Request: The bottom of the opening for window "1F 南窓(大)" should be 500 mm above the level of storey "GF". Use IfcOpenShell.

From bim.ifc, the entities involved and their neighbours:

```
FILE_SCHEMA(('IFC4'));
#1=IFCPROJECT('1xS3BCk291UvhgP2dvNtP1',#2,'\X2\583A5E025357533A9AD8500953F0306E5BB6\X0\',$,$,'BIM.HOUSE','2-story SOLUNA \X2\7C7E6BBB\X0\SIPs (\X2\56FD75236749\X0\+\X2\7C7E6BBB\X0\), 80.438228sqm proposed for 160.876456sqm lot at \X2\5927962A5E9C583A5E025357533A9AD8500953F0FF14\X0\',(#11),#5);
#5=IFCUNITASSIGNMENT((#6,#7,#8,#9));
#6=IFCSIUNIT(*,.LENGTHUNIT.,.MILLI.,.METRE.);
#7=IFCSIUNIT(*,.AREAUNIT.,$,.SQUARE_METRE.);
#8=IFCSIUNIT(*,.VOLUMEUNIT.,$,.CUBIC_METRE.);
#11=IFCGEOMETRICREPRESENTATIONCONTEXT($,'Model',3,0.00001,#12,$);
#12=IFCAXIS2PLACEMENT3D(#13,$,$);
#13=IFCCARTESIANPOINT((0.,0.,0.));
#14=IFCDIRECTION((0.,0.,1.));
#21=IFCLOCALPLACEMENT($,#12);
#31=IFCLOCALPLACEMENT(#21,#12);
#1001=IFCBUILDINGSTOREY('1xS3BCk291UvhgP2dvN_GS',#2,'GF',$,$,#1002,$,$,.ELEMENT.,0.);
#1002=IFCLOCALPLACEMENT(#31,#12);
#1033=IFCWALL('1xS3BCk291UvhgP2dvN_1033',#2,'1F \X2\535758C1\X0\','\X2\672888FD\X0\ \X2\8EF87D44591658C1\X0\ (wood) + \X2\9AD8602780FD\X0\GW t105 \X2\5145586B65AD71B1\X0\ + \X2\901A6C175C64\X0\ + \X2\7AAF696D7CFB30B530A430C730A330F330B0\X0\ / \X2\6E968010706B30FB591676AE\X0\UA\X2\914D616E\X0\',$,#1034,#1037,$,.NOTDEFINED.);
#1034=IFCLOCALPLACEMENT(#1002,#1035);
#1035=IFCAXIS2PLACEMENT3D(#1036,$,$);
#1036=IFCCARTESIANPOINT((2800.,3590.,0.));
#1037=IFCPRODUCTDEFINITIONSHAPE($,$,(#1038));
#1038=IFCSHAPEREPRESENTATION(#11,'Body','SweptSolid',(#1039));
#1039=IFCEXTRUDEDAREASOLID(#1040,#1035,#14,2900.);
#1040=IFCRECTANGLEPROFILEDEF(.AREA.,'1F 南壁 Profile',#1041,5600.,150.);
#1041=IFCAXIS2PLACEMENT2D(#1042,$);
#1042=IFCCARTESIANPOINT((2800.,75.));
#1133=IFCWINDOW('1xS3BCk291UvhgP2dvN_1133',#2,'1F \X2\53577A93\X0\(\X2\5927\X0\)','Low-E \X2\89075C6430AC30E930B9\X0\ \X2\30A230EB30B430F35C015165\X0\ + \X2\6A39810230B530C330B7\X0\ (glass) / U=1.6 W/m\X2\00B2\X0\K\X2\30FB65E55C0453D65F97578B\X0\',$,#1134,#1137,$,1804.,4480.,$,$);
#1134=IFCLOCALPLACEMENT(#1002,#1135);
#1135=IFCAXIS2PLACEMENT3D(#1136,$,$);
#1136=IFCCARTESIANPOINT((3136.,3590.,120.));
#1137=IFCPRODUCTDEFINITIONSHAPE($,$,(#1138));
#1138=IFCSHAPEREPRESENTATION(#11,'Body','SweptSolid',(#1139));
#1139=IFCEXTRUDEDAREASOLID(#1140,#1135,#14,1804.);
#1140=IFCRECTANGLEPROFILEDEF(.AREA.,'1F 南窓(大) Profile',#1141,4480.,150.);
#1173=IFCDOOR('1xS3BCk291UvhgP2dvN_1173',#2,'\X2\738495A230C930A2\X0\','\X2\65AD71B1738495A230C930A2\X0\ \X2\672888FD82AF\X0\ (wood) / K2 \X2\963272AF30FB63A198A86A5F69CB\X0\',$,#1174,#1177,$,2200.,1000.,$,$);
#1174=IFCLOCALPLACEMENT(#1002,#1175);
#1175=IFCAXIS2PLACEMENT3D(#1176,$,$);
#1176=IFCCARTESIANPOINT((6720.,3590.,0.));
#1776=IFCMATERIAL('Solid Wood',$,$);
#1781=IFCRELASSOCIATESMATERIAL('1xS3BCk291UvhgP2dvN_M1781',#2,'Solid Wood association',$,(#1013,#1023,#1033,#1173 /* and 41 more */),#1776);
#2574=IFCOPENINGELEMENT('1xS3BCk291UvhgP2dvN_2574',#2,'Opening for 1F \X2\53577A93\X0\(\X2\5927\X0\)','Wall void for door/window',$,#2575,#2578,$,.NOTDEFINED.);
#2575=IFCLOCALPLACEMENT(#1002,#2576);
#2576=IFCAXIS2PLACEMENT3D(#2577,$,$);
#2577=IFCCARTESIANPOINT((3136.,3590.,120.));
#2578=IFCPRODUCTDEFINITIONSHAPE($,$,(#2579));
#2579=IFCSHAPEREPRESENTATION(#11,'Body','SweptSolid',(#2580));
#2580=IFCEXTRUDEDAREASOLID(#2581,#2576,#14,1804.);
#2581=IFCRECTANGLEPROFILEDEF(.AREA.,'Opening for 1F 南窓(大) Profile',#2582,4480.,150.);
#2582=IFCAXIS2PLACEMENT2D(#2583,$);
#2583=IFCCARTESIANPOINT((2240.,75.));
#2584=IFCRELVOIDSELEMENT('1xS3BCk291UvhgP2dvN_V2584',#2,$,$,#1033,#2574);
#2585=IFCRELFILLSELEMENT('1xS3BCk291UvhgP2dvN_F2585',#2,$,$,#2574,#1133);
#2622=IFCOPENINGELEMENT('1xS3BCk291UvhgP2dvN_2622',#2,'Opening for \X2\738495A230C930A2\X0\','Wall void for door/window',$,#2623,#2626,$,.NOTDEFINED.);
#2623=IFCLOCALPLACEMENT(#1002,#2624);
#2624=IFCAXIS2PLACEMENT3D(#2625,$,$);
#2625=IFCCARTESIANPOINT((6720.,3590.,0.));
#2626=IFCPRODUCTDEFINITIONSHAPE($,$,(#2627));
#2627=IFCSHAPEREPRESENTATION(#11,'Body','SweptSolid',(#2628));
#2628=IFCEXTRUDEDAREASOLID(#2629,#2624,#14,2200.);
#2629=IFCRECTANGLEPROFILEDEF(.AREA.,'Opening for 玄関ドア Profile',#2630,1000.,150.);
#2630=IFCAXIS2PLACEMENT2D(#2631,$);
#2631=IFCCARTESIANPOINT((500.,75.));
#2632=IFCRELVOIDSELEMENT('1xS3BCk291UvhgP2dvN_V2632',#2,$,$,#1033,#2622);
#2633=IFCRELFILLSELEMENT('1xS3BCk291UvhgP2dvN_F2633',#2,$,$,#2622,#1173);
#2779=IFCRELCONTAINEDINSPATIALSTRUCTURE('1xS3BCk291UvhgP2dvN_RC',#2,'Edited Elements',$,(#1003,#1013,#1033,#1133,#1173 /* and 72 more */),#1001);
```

```python
import numpy as np
import ifcopenshell
import ifcopenshell.api.geometry
import ifcopenshell.geom
import ifcopenshell.util.element
import ifcopenshell.util.placement
import ifcopenshell.util.shape
import ifcopenshell.util.unit

model = ifcopenshell.open("bim.ifc")
unit_scale = ifcopenshell.util.unit.calculate_unit_scale(model)

window = model.by_guid("1xS3BCk291UvhgP2dvN_1133")
opening = window.FillsVoids[0].RelatingOpeningElement
storey = ifcopenshell.util.element.get_container(window, ifc_class="IfcBuildingStorey")
level = ifcopenshell.util.placement.get_local_placement(storey.ObjectPlacement)[2, 3]

# The opening's origin need not be at the sill, so measure its lowest point.
shape = ifcopenshell.geom.create_shape(ifcopenshell.geom.settings(), opening)
bottom = ifcopenshell.util.shape.get_shape_bottom_elevation(shape, shape.geometry) / unit_scale
dz = level + 0.5 / unit_scale - bottom

shift = np.array([0.0, 0.0, dz])
# The window is not placed relative to its opening, so move both.
for product in (opening, window):
    matrix = ifcopenshell.util.placement.get_local_placement(product.ObjectPlacement)
    matrix[:3, 3] += shift
    ifcopenshell.api.geometry.edit_object_placement(model, product=product, matrix=matrix, is_si=False)

print(f"moved by {dz * unit_scale:+.3f} m")

model.write("bim_updated.ifc")
```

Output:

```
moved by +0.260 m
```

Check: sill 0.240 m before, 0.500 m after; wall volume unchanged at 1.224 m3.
